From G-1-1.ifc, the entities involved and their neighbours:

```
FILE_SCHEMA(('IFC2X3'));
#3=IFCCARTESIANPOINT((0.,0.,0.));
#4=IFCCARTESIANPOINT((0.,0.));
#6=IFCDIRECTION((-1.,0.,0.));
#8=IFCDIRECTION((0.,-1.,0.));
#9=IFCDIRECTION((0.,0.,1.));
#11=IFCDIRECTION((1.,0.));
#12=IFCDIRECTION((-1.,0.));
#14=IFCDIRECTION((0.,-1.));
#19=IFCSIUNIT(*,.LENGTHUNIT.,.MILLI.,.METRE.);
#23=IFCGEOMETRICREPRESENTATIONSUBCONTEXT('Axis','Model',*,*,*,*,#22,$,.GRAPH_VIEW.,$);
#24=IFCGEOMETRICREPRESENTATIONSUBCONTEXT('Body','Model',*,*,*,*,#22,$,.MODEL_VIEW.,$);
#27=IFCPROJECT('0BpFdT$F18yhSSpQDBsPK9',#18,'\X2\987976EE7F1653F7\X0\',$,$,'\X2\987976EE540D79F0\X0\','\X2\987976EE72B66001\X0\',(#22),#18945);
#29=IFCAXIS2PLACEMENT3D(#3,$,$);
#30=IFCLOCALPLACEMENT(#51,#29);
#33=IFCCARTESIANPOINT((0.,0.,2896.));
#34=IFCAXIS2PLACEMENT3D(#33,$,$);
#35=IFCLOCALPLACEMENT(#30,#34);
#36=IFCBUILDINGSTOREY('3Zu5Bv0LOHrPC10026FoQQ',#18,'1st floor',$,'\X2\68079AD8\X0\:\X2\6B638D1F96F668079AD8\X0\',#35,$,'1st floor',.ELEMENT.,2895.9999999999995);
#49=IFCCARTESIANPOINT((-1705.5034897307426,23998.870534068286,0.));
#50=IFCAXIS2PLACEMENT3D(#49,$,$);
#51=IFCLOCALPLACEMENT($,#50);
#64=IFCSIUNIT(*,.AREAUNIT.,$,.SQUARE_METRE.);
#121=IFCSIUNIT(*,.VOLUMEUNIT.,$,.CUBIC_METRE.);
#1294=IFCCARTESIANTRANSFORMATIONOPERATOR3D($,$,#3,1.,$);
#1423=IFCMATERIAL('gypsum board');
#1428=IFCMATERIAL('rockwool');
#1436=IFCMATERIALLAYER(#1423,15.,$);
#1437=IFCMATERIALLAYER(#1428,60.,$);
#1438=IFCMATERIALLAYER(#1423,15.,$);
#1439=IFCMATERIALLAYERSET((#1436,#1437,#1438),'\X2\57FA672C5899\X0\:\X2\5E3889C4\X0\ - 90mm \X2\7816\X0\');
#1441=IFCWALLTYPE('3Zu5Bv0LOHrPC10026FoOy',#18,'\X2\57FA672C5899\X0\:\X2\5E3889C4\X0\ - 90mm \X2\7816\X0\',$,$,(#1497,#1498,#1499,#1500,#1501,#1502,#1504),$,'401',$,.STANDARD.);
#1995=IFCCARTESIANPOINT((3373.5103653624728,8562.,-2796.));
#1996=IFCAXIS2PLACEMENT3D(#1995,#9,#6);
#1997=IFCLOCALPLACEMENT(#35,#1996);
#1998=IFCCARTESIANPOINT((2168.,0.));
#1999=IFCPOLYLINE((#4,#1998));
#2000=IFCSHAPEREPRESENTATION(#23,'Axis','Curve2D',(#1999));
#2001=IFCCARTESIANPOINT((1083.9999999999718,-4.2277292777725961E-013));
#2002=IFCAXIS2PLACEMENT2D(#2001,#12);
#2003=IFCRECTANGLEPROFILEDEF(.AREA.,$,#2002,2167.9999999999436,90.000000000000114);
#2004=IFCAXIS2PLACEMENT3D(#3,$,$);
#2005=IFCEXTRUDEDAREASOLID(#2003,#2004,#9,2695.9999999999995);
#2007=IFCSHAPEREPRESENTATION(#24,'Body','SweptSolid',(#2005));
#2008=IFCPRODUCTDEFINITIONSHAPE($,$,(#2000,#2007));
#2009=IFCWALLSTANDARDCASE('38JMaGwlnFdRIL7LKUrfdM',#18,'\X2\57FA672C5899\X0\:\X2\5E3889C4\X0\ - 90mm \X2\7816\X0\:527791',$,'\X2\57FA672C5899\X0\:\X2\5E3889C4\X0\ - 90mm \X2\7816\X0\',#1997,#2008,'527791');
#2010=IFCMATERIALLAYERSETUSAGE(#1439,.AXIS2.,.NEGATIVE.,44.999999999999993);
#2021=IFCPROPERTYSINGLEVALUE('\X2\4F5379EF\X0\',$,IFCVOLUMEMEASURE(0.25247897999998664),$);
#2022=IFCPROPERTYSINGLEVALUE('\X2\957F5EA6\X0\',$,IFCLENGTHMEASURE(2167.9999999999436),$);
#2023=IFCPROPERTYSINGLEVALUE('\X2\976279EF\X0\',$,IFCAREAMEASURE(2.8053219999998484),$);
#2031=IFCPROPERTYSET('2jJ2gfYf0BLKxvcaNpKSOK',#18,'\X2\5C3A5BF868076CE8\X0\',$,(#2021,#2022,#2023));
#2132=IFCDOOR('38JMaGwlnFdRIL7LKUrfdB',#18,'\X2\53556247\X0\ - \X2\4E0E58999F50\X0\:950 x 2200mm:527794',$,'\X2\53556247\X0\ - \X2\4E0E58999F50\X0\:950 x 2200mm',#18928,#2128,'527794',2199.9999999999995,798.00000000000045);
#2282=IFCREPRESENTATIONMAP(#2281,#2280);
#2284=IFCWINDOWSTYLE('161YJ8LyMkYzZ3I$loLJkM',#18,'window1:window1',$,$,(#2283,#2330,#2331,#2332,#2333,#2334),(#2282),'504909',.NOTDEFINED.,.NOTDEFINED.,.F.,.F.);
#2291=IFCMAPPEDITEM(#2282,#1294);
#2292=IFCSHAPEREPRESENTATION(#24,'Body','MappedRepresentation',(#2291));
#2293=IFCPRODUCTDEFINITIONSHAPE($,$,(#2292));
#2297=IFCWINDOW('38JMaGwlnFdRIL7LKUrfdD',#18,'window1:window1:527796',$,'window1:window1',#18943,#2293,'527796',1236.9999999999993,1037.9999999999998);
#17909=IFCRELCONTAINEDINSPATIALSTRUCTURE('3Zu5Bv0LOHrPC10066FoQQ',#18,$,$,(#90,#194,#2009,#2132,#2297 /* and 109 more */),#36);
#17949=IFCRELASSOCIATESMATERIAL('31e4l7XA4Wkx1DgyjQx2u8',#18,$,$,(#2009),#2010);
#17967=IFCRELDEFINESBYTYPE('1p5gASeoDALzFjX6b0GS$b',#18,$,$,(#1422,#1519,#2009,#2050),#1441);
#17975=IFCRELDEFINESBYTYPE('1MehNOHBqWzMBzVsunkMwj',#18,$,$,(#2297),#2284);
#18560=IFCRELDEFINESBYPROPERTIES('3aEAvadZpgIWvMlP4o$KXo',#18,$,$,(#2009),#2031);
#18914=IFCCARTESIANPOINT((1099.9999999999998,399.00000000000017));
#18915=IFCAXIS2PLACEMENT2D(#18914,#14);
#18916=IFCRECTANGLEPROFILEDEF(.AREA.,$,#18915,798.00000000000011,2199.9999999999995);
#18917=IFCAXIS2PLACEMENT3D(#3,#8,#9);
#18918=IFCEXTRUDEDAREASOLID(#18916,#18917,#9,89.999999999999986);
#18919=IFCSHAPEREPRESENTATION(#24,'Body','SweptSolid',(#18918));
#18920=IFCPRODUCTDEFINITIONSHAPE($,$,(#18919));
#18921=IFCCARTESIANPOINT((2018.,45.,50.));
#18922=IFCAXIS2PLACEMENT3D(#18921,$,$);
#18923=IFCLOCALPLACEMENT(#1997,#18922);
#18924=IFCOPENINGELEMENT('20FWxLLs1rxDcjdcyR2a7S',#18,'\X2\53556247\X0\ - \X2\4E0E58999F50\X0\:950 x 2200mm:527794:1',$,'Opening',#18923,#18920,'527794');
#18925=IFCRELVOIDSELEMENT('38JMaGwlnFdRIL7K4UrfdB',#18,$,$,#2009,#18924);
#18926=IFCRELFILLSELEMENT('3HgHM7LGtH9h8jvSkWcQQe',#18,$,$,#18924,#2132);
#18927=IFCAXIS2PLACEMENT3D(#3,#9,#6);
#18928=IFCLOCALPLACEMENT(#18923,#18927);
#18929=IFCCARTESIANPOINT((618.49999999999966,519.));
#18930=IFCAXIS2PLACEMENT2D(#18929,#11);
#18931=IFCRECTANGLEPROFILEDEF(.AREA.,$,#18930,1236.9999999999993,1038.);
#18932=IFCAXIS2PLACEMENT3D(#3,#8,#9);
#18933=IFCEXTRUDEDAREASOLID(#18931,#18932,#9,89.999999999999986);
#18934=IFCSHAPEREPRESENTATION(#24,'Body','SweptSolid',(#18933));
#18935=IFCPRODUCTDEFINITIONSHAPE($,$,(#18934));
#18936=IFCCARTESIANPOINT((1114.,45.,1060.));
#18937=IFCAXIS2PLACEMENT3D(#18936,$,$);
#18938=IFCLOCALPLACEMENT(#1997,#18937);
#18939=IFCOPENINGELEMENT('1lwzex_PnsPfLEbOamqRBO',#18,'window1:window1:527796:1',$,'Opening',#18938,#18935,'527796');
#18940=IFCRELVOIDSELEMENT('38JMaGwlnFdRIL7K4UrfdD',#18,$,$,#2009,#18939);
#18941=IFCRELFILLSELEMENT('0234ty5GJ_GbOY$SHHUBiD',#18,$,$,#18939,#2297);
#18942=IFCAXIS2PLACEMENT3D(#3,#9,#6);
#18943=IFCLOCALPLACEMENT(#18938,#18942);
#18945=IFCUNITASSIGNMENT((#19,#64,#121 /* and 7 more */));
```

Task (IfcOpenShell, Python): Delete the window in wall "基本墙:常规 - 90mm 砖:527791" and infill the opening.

```python
import ifcopenshell
import ifcopenshell.api.feature
import ifcopenshell.api.pset
import ifcopenshell.api.root
import ifcopenshell.geom
import ifcopenshell.util.element
import ifcopenshell.util.shape
import ifcopenshell.util.unit

model = ifcopenshell.open("G-1-1.ifc")
area_scale = ifcopenshell.util.unit.calculate_unit_scale(model, "AREAUNIT")
volume_scale = ifcopenshell.util.unit.calculate_unit_scale(model, "VOLUMEUNIT")
settings = ifcopenshell.geom.settings()


def volume(element):
    """Net volume in cubic metres, openings subtracted."""
    shape = ifcopenshell.geom.create_shape(settings, element)
    return ifcopenshell.util.shape.get_volume(shape.geometry)


window = model.by_id(2297)
opening = window.FillsVoids[0].RelatingOpeningElement
wall = opening.VoidsElements[0].RelatingBuildingElement
before = volume(wall)

ifcopenshell.api.root.remove_product(model, product=window)
ifcopenshell.api.feature.remove_feature(model, feature=opening)

after = volume(wall)
thickness = 0.09  # wall thickness in metres

# Update the wall's stored quantities.
pset = model.by_id(ifcopenshell.util.element.get_pset(wall, "尺寸标注", should_inherit=False)["id"])
ifcopenshell.api.pset.edit_pset(model, pset=pset, properties={
    "体积": model.create_entity("IfcVolumeMeasure", after / volume_scale),
    "面积": model.create_entity("IfcAreaMeasure", after / thickness / area_scale),
})

print(f"wall volume {before:.3f} -> {after:.3f} m3")

model.write("G-1-1-out.ifc")
```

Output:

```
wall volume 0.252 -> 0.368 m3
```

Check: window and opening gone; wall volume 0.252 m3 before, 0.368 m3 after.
